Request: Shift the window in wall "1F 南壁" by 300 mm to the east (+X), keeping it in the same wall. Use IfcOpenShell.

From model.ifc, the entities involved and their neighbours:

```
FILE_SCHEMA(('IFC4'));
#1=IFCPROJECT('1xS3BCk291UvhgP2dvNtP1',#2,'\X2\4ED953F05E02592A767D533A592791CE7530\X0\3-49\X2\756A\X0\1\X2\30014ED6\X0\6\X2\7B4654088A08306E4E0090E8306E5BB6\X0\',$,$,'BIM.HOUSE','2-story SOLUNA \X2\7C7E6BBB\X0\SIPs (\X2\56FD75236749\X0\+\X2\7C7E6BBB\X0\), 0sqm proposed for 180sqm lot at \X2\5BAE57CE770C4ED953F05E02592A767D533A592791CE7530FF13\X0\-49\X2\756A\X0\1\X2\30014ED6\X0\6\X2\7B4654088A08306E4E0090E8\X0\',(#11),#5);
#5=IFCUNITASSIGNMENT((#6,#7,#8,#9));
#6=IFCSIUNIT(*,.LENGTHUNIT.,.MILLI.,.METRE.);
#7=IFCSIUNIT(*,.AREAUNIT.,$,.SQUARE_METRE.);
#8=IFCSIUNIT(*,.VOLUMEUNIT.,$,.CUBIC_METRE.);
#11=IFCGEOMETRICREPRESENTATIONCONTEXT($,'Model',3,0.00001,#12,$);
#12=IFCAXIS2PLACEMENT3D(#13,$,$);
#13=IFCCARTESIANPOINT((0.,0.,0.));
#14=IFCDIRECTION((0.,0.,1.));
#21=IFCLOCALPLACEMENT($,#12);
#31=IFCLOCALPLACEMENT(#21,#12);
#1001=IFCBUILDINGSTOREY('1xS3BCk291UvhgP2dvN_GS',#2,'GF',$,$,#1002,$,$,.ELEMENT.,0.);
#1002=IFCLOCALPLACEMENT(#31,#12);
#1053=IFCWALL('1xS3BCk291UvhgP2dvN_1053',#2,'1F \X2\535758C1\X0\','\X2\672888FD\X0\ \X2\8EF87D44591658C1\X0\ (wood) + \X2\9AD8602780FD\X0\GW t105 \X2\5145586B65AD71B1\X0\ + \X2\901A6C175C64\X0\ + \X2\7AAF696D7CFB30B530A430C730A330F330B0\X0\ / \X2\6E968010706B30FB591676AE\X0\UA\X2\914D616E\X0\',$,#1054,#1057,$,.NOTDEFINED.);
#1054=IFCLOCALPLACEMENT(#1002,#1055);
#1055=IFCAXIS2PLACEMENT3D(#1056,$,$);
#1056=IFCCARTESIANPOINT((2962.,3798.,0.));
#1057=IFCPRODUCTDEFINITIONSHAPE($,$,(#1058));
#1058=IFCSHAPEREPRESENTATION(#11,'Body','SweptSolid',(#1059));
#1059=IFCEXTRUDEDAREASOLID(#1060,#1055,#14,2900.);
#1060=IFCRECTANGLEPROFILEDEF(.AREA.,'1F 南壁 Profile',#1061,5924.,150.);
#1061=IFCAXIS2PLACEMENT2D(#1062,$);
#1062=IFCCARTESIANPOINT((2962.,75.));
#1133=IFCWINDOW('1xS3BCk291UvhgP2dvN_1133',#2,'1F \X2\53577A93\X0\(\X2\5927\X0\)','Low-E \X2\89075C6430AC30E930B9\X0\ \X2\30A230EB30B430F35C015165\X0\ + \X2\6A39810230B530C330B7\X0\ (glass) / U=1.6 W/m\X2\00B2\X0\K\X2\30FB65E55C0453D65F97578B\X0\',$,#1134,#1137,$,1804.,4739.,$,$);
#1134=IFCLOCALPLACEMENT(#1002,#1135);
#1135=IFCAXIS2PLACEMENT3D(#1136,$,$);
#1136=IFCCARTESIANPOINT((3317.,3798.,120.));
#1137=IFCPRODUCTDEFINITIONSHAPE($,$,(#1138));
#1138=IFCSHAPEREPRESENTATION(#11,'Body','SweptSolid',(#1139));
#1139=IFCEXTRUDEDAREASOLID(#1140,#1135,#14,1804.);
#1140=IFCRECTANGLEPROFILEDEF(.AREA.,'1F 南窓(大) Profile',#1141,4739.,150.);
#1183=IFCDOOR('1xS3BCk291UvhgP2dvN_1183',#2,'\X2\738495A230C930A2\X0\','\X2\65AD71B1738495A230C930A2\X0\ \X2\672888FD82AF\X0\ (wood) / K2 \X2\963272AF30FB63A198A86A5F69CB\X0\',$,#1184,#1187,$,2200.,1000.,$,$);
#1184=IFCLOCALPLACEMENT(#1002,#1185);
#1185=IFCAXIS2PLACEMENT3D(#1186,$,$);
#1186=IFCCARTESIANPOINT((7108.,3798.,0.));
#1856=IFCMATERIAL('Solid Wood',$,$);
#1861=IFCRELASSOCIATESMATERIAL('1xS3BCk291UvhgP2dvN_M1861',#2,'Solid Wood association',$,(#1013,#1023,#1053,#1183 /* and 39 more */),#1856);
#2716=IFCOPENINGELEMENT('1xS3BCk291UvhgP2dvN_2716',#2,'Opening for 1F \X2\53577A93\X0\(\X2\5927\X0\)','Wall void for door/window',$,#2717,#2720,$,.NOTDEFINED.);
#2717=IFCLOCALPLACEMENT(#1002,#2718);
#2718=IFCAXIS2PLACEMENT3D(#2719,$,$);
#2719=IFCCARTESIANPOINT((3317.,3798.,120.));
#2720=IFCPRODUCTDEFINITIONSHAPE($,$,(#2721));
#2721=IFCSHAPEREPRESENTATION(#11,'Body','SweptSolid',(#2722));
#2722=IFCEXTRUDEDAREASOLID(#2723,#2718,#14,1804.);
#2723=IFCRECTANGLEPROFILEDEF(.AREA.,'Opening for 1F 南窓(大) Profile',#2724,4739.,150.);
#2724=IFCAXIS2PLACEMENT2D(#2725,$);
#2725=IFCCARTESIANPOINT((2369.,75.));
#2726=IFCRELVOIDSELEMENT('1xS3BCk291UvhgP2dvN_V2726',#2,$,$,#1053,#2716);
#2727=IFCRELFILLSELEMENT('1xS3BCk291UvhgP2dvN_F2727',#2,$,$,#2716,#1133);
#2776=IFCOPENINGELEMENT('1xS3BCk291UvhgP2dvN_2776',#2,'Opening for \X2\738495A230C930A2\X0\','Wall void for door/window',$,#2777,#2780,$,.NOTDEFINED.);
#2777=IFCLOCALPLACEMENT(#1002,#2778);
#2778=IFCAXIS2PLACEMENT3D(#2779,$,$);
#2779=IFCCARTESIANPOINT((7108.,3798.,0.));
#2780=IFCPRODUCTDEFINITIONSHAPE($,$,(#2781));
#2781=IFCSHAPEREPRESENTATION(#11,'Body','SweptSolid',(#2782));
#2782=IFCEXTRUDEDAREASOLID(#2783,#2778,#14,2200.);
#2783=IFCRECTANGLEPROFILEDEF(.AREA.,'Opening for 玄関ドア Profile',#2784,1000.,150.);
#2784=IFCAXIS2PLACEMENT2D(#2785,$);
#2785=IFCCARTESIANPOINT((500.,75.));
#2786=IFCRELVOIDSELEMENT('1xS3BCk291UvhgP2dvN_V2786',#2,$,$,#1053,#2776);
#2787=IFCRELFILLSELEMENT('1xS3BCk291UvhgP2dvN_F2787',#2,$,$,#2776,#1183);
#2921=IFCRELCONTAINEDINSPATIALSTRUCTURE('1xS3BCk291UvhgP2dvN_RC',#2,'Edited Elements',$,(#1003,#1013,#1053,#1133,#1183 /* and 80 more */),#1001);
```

```python
import ifcopenshell
import ifcopenshell.api.geometry
import ifcopenshell.util.placement
import ifcopenshell.util.unit

model = ifcopenshell.open("model.ifc")
unit_scale = ifcopenshell.util.unit.calculate_unit_scale(model)

window = model.by_id(1133)
opening = window.FillsVoids[0].RelatingOpeningElement
wall = opening.VoidsElements[0].RelatingBuildingElement

wall_matrix = ifcopenshell.util.placement.get_local_placement(wall.ObjectPlacement)
shift = wall_matrix[:3, 0] * 0.3 / unit_scale
before = ifcopenshell.util.placement.get_local_placement(window.ObjectPlacement)[:3, 3].copy()

# The window is not placed relative to its opening, so move both.
for product in (opening, window):
    matrix = ifcopenshell.util.placement.get_local_placement(product.ObjectPlacement)
    matrix[:3, 3] += shift
    ifcopenshell.api.geometry.edit_object_placement(model, product=product, matrix=matrix, is_si=False)

after = ifcopenshell.util.placement.get_local_placement(window.ObjectPlacement)[:3, 3]
print("window moved by", (after - before).round(3) + 0.0)

model.write("model_v2.ifc")
```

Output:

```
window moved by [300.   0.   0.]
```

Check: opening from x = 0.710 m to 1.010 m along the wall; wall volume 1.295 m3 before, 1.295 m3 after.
